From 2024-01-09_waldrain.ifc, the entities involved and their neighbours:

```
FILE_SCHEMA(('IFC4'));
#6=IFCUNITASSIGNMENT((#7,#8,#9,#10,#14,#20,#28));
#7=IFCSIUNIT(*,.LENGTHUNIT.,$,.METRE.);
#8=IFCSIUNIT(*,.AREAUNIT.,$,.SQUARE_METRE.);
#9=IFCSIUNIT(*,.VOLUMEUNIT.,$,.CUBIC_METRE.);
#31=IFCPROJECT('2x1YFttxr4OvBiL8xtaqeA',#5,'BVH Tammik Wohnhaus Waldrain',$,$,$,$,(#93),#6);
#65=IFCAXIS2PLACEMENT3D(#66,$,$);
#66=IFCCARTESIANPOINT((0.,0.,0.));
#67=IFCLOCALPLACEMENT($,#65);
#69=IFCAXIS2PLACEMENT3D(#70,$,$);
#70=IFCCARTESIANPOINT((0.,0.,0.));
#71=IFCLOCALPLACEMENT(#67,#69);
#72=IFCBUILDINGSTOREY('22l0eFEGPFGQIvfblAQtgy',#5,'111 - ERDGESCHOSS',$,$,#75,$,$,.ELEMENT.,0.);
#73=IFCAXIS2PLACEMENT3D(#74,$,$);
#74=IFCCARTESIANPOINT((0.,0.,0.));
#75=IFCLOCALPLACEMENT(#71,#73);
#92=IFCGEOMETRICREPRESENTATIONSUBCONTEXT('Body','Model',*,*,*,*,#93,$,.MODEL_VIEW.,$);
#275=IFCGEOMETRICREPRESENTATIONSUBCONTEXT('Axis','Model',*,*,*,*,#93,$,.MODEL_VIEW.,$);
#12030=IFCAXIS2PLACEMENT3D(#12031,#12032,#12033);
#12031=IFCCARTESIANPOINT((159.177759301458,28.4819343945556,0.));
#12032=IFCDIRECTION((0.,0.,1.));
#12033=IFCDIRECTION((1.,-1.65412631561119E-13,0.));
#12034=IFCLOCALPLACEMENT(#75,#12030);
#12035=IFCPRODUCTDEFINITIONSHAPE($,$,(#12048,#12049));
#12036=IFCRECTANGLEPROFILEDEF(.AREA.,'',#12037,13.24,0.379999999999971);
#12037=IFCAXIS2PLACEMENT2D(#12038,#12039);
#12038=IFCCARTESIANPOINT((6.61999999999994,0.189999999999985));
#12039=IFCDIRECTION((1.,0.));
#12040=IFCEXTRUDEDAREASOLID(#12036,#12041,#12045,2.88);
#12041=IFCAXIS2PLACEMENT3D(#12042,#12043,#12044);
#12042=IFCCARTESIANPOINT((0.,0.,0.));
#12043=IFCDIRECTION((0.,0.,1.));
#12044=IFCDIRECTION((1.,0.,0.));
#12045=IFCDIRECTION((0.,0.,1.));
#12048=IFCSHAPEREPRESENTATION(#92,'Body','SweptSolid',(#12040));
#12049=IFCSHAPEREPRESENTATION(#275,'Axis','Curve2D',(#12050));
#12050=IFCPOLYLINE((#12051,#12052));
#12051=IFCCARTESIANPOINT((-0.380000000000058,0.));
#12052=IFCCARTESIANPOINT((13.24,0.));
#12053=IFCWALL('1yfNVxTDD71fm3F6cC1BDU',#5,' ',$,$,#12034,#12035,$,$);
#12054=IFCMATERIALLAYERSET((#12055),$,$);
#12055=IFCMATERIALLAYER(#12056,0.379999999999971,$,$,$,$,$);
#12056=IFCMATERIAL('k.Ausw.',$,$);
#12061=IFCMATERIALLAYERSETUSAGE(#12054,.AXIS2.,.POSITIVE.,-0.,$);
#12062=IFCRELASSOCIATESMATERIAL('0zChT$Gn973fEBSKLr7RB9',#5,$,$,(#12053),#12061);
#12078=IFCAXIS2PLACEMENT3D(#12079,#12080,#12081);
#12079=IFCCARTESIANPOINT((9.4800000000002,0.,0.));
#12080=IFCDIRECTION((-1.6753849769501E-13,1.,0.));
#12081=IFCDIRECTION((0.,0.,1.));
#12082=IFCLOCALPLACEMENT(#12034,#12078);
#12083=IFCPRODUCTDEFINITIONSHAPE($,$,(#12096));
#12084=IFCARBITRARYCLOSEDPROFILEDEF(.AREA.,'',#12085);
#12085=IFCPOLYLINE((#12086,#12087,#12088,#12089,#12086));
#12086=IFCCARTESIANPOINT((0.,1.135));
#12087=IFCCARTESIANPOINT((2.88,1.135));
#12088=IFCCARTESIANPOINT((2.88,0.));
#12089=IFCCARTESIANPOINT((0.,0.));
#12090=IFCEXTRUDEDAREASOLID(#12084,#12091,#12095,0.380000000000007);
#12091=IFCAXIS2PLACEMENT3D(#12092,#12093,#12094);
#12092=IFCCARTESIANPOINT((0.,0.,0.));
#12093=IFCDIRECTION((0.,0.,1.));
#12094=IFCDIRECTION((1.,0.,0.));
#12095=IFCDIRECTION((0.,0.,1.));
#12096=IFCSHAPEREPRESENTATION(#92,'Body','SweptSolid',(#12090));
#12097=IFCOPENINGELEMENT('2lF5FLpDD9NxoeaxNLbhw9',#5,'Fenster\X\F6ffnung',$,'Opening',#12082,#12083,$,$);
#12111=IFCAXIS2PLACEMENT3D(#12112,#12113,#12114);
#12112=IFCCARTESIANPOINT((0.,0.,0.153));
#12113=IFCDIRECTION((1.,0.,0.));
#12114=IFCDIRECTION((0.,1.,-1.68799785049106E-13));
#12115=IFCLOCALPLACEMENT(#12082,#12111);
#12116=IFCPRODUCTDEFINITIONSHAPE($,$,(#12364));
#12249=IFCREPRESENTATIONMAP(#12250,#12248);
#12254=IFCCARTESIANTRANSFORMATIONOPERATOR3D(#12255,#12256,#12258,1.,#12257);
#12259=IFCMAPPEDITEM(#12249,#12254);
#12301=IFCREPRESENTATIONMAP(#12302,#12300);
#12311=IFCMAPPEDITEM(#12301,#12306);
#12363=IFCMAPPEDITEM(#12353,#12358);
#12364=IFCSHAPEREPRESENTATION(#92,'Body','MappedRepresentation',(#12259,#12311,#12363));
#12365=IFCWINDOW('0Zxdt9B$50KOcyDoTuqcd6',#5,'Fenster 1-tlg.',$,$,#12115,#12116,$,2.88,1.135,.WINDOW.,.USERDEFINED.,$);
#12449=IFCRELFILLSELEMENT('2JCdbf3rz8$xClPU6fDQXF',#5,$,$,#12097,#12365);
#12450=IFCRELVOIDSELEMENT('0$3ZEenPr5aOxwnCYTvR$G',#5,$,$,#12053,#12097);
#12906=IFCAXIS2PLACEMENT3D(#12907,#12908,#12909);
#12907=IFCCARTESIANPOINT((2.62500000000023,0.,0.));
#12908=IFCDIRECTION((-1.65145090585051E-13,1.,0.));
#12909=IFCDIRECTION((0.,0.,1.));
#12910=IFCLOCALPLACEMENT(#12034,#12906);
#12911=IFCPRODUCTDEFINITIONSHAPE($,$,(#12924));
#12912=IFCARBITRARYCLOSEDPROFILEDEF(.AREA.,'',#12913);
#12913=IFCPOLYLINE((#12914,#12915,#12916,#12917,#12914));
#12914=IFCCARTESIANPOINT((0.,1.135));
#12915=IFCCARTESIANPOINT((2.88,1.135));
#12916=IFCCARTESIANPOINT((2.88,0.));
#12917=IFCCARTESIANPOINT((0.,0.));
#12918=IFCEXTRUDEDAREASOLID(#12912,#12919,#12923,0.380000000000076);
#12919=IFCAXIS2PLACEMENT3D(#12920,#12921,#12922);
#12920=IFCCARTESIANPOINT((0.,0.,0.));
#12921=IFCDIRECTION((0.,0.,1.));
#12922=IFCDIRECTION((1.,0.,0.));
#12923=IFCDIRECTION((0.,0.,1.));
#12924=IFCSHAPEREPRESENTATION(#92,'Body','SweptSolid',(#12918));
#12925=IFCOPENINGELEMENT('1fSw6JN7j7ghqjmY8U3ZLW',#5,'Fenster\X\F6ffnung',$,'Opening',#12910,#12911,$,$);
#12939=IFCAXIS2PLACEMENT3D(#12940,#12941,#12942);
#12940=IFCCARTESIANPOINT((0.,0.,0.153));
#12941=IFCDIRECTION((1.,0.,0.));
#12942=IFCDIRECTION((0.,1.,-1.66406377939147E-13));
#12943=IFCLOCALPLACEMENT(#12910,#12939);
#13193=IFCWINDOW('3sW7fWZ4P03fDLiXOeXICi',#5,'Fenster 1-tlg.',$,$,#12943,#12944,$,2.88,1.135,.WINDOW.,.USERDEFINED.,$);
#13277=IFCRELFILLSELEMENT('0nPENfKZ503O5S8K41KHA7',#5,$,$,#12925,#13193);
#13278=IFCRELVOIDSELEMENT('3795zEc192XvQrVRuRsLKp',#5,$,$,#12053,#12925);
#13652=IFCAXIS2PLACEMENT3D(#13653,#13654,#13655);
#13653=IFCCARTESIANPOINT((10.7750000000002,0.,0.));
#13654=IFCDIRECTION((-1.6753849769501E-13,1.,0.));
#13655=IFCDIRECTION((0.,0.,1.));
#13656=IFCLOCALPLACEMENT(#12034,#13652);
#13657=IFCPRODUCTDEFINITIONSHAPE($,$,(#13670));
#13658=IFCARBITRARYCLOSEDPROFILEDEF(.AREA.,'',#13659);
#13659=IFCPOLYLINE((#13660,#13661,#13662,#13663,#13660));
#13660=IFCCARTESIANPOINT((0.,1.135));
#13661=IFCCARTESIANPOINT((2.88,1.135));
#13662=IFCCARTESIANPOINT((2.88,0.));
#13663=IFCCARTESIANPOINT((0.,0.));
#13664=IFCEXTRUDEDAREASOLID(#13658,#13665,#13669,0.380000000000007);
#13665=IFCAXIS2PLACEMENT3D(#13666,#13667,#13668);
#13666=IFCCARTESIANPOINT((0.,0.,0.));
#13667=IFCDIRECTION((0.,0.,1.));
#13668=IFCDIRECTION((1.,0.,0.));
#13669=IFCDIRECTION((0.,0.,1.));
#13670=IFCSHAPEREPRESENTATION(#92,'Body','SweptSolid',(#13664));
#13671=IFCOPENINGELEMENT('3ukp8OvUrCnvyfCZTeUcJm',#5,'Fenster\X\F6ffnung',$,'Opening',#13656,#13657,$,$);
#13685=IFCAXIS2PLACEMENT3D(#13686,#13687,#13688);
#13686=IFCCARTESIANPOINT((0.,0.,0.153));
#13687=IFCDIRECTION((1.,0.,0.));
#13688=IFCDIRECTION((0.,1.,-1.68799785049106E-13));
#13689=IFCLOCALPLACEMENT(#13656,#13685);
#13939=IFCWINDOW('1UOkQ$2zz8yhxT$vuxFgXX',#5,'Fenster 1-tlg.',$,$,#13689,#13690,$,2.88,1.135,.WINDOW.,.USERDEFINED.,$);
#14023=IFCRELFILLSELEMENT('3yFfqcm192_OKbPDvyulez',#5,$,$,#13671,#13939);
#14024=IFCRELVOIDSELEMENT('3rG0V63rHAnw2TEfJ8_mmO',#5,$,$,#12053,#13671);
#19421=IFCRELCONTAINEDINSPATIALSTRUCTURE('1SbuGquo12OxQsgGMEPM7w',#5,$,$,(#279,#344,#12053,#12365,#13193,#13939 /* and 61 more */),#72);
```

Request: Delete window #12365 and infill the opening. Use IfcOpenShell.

```python
import ifcopenshell
import ifcopenshell.api.feature
import ifcopenshell.api.root
import ifcopenshell.geom
import ifcopenshell.util.shape

model = ifcopenshell.open("2024-01-09_waldrain.ifc")
settings = ifcopenshell.geom.settings()


def volume(element):
    """Net volume in cubic metres, openings subtracted."""
    shape = ifcopenshell.geom.create_shape(settings, element)
    return ifcopenshell.util.shape.get_volume(shape.geometry)


window = model.by_id(12365)
opening = window.FillsVoids[0].RelatingOpeningElement
wall = opening.VoidsElements[0].RelatingBuildingElement
before = volume(wall)

ifcopenshell.api.root.remove_product(model, product=window)
ifcopenshell.api.feature.remove_feature(model, feature=opening)

after = volume(wall)

print(f"wall volume {before:.3f} -> {after:.3f} m3")

model.write("2024-01-09_waldrain_rev.ifc")
```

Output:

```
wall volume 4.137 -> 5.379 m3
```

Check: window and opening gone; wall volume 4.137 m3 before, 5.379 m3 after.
